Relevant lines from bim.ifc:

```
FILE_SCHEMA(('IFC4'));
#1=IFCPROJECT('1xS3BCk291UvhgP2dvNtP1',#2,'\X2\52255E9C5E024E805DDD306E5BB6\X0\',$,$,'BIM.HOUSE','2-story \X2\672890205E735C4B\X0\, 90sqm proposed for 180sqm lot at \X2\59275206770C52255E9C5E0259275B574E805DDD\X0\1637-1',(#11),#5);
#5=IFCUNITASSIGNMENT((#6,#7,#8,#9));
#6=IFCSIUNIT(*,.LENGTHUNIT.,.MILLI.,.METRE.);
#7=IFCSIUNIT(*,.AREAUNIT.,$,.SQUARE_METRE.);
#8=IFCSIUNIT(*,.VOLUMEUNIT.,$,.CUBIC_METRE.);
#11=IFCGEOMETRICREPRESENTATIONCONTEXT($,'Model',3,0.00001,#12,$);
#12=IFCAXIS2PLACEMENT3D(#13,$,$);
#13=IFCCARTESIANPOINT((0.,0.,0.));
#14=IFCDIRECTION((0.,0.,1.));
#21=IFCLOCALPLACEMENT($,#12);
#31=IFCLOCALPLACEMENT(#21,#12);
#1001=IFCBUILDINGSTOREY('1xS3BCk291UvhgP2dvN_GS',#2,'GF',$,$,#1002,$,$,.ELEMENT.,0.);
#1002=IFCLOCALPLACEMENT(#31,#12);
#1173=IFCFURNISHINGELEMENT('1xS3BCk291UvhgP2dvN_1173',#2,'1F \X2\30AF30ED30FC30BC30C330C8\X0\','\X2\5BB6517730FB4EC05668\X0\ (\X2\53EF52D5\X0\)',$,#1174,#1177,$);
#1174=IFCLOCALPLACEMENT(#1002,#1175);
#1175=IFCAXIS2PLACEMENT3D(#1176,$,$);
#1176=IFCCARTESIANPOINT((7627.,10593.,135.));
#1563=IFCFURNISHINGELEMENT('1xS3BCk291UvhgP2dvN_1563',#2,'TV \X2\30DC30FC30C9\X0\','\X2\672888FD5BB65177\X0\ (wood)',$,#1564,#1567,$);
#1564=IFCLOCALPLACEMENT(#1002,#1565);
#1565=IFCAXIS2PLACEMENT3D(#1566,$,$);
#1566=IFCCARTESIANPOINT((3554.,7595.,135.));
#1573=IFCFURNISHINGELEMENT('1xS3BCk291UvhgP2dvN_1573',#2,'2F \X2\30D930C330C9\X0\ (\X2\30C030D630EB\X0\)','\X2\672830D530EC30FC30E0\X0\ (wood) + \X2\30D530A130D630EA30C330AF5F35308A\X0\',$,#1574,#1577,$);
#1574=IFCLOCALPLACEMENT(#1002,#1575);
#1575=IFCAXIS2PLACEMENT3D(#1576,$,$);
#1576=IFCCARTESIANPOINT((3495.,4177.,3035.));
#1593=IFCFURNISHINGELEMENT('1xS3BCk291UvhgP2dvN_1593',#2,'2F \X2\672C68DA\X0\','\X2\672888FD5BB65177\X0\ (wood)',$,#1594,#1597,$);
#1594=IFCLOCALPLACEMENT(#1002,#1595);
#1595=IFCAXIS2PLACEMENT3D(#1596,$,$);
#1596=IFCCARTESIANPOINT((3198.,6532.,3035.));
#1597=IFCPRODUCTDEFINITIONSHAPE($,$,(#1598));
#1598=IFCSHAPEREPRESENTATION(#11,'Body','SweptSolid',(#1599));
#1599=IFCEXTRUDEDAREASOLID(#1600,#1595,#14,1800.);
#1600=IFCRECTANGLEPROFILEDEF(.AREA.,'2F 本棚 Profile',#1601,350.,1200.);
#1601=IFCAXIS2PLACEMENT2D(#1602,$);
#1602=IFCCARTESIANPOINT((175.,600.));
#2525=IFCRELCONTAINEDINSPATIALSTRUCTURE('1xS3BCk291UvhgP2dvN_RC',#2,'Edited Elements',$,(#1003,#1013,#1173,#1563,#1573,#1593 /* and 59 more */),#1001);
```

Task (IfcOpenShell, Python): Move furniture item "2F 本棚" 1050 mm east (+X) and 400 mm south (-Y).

```python
import ifcopenshell
import ifcopenshell.api.geometry
import ifcopenshell.util.placement
import ifcopenshell.util.unit

model = ifcopenshell.open("bim.ifc")
unit_scale = ifcopenshell.util.unit.calculate_unit_scale(model)

item = model.by_guid("1xS3BCk291UvhgP2dvN_1593")
matrix = ifcopenshell.util.placement.get_local_placement(item.ObjectPlacement)
matrix[0, 3] += 1.05 / unit_scale
matrix[1, 3] -= 0.4 / unit_scale
ifcopenshell.api.geometry.edit_object_placement(model, product=item, matrix=matrix, is_si=False)

print(ifcopenshell.util.placement.get_local_placement(item.ObjectPlacement).round(3) + 0.0)

model.write("bim-out.ifc")
```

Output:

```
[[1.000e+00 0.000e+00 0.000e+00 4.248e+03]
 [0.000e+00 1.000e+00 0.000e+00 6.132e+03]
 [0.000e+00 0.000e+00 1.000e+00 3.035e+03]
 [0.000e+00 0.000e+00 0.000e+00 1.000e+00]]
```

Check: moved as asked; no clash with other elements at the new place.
